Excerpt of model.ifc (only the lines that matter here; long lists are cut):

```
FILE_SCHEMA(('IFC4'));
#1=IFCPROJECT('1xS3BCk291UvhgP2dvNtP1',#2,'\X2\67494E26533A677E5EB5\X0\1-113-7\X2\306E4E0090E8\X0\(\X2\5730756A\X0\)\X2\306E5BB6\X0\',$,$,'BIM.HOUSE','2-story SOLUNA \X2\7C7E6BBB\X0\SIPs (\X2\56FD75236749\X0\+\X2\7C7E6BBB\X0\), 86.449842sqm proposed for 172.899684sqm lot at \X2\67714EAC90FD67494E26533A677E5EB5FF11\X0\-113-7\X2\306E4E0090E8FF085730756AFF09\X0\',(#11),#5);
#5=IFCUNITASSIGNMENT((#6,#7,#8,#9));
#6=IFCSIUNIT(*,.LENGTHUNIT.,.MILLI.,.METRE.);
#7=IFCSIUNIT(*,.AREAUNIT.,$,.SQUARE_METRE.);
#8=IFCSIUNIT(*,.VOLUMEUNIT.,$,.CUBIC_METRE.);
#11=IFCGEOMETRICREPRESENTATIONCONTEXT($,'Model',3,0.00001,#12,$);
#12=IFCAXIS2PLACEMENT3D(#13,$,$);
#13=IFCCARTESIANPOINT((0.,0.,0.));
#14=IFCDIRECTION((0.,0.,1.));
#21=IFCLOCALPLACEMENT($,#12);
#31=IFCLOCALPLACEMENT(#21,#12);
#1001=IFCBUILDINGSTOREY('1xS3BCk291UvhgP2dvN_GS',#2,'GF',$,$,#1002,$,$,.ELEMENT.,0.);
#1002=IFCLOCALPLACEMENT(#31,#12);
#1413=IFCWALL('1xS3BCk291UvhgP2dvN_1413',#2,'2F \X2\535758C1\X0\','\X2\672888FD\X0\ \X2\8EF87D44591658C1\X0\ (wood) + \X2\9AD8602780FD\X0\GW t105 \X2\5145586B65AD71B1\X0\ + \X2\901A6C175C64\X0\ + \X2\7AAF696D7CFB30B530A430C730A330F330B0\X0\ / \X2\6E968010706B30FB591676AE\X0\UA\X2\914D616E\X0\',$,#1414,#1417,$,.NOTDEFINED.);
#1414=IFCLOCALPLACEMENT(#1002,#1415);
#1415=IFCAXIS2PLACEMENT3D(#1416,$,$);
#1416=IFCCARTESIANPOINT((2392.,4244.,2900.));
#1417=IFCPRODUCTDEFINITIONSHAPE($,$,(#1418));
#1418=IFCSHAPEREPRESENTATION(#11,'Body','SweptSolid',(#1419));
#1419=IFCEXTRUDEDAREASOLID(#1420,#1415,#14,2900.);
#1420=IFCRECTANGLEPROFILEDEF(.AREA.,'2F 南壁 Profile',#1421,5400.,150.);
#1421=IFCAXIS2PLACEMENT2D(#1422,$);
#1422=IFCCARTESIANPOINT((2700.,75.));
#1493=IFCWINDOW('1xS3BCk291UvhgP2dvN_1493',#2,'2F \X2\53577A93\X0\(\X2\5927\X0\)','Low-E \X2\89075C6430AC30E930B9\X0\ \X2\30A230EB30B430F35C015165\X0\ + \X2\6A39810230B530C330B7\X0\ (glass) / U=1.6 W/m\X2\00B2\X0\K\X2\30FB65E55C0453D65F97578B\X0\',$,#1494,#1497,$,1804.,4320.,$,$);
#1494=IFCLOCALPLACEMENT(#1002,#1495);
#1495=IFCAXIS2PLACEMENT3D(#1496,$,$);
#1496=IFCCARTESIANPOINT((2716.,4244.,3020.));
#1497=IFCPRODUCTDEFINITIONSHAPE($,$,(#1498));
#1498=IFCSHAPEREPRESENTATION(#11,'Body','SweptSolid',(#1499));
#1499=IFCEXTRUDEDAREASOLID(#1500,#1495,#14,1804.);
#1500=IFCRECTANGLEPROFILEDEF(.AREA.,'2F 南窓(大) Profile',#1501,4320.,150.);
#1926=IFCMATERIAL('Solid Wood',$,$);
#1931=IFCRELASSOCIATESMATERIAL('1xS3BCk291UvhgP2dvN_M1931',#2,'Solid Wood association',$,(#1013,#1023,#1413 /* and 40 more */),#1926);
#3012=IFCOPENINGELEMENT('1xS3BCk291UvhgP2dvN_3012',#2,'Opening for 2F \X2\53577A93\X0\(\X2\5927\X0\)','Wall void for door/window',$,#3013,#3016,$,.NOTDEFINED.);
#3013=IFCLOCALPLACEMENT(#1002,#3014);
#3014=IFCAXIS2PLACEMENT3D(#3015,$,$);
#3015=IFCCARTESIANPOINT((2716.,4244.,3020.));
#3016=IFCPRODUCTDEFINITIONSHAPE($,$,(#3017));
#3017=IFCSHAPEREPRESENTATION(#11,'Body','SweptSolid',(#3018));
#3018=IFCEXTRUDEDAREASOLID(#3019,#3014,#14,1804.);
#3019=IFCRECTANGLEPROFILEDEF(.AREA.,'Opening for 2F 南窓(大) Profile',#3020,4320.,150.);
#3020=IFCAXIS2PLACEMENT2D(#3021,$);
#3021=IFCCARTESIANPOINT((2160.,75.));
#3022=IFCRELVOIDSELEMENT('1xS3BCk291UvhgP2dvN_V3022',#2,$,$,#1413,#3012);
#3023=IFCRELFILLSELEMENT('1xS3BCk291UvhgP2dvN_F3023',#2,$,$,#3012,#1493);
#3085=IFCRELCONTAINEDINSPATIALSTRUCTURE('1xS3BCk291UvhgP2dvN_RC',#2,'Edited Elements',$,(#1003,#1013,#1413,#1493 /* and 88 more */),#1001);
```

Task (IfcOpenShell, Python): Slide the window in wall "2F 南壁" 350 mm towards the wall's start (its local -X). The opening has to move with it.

```python
import ifcopenshell
import ifcopenshell.api.geometry
import ifcopenshell.util.placement

model = ifcopenshell.open("model.ifc")

window = model.by_guid("1xS3BCk291UvhgP2dvN_1493")
opening = window.FillsVoids[0].RelatingOpeningElement
wall = opening.VoidsElements[0].RelatingBuildingElement

wall_matrix = ifcopenshell.util.placement.get_local_placement(wall.ObjectPlacement)
shift = wall_matrix[:3, 0] * -350.0
before = ifcopenshell.util.placement.get_local_placement(window.ObjectPlacement)[:3, 3].copy()

# The window is not placed relative to its opening, so move both.
for product in (opening, window):
    matrix = ifcopenshell.util.placement.get_local_placement(product.ObjectPlacement)
    matrix[:3, 3] += shift
    ifcopenshell.api.geometry.edit_object_placement(model, product=product, matrix=matrix, is_si=False)

after = ifcopenshell.util.placement.get_local_placement(window.ObjectPlacement)[:3, 3]
print("window moved by", (after - before).round(3) + 0.0)

model.write("model_rev.ifc")
```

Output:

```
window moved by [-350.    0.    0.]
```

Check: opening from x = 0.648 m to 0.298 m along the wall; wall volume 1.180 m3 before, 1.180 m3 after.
